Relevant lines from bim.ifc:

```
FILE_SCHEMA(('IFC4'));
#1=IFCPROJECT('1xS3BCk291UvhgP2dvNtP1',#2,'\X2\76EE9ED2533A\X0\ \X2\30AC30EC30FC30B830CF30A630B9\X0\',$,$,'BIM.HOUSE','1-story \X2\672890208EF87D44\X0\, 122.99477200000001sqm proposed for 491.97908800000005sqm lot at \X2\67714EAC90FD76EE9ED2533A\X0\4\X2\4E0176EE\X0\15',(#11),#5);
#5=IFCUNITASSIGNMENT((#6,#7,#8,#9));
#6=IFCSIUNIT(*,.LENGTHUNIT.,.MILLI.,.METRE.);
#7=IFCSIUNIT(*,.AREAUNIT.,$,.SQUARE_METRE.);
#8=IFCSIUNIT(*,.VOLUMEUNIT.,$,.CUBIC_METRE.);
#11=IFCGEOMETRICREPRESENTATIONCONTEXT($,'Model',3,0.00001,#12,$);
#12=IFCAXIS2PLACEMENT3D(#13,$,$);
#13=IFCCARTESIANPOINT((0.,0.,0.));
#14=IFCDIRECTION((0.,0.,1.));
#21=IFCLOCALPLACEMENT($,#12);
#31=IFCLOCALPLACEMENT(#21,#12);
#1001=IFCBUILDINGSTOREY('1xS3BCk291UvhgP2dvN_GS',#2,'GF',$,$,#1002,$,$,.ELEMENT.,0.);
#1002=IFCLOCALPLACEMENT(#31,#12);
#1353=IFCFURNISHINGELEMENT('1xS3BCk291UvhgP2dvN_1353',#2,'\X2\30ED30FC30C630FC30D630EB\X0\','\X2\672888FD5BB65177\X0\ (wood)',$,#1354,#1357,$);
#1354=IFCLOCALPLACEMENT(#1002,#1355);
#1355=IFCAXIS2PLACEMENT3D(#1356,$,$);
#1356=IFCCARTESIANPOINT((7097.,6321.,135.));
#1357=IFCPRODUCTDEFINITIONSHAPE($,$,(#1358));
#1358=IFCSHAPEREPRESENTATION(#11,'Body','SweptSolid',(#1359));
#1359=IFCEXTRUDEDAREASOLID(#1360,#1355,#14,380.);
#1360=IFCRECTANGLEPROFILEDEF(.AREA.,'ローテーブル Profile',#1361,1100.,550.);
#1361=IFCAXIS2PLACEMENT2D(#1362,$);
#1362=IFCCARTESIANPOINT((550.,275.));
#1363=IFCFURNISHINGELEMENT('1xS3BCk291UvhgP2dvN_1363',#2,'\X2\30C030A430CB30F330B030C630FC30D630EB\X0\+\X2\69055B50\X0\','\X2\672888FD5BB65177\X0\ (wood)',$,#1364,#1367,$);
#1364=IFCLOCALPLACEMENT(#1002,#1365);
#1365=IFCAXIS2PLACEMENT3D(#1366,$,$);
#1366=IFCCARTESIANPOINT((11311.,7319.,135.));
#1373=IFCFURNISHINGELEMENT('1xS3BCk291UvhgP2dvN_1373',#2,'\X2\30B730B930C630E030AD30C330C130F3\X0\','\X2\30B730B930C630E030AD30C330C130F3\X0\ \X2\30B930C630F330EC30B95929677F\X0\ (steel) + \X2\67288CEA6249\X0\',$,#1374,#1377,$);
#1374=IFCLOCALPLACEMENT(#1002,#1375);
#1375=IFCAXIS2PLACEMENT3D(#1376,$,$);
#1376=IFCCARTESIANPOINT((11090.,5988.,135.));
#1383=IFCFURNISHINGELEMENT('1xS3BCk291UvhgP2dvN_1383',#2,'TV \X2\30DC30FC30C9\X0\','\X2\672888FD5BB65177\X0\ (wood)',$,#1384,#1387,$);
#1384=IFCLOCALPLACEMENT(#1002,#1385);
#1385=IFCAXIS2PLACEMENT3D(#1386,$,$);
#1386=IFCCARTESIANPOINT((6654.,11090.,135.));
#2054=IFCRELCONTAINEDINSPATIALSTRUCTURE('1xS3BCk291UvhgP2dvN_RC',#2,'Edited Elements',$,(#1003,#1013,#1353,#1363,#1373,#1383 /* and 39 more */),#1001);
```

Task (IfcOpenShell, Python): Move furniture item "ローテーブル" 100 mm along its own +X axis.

```python
import ifcopenshell
import ifcopenshell.api.geometry
import ifcopenshell.util.placement
import ifcopenshell.util.unit

model = ifcopenshell.open("bim.ifc")
unit_scale = ifcopenshell.util.unit.calculate_unit_scale(model)

item = model.by_guid("1xS3BCk291UvhgP2dvN_1353")
matrix = ifcopenshell.util.placement.get_local_placement(item.ObjectPlacement)
matrix[:3, 3] += matrix[:3, 0] * 0.1 / unit_scale
ifcopenshell.api.geometry.edit_object_placement(model, product=item, matrix=matrix, is_si=False)

print(ifcopenshell.util.placement.get_local_placement(item.ObjectPlacement).round(3) + 0.0)

model.write("bim_rev.ifc")
```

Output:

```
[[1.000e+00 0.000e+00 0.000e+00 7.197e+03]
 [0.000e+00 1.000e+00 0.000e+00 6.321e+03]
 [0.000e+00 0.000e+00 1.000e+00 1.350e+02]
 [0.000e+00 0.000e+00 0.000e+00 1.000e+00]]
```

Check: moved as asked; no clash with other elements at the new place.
